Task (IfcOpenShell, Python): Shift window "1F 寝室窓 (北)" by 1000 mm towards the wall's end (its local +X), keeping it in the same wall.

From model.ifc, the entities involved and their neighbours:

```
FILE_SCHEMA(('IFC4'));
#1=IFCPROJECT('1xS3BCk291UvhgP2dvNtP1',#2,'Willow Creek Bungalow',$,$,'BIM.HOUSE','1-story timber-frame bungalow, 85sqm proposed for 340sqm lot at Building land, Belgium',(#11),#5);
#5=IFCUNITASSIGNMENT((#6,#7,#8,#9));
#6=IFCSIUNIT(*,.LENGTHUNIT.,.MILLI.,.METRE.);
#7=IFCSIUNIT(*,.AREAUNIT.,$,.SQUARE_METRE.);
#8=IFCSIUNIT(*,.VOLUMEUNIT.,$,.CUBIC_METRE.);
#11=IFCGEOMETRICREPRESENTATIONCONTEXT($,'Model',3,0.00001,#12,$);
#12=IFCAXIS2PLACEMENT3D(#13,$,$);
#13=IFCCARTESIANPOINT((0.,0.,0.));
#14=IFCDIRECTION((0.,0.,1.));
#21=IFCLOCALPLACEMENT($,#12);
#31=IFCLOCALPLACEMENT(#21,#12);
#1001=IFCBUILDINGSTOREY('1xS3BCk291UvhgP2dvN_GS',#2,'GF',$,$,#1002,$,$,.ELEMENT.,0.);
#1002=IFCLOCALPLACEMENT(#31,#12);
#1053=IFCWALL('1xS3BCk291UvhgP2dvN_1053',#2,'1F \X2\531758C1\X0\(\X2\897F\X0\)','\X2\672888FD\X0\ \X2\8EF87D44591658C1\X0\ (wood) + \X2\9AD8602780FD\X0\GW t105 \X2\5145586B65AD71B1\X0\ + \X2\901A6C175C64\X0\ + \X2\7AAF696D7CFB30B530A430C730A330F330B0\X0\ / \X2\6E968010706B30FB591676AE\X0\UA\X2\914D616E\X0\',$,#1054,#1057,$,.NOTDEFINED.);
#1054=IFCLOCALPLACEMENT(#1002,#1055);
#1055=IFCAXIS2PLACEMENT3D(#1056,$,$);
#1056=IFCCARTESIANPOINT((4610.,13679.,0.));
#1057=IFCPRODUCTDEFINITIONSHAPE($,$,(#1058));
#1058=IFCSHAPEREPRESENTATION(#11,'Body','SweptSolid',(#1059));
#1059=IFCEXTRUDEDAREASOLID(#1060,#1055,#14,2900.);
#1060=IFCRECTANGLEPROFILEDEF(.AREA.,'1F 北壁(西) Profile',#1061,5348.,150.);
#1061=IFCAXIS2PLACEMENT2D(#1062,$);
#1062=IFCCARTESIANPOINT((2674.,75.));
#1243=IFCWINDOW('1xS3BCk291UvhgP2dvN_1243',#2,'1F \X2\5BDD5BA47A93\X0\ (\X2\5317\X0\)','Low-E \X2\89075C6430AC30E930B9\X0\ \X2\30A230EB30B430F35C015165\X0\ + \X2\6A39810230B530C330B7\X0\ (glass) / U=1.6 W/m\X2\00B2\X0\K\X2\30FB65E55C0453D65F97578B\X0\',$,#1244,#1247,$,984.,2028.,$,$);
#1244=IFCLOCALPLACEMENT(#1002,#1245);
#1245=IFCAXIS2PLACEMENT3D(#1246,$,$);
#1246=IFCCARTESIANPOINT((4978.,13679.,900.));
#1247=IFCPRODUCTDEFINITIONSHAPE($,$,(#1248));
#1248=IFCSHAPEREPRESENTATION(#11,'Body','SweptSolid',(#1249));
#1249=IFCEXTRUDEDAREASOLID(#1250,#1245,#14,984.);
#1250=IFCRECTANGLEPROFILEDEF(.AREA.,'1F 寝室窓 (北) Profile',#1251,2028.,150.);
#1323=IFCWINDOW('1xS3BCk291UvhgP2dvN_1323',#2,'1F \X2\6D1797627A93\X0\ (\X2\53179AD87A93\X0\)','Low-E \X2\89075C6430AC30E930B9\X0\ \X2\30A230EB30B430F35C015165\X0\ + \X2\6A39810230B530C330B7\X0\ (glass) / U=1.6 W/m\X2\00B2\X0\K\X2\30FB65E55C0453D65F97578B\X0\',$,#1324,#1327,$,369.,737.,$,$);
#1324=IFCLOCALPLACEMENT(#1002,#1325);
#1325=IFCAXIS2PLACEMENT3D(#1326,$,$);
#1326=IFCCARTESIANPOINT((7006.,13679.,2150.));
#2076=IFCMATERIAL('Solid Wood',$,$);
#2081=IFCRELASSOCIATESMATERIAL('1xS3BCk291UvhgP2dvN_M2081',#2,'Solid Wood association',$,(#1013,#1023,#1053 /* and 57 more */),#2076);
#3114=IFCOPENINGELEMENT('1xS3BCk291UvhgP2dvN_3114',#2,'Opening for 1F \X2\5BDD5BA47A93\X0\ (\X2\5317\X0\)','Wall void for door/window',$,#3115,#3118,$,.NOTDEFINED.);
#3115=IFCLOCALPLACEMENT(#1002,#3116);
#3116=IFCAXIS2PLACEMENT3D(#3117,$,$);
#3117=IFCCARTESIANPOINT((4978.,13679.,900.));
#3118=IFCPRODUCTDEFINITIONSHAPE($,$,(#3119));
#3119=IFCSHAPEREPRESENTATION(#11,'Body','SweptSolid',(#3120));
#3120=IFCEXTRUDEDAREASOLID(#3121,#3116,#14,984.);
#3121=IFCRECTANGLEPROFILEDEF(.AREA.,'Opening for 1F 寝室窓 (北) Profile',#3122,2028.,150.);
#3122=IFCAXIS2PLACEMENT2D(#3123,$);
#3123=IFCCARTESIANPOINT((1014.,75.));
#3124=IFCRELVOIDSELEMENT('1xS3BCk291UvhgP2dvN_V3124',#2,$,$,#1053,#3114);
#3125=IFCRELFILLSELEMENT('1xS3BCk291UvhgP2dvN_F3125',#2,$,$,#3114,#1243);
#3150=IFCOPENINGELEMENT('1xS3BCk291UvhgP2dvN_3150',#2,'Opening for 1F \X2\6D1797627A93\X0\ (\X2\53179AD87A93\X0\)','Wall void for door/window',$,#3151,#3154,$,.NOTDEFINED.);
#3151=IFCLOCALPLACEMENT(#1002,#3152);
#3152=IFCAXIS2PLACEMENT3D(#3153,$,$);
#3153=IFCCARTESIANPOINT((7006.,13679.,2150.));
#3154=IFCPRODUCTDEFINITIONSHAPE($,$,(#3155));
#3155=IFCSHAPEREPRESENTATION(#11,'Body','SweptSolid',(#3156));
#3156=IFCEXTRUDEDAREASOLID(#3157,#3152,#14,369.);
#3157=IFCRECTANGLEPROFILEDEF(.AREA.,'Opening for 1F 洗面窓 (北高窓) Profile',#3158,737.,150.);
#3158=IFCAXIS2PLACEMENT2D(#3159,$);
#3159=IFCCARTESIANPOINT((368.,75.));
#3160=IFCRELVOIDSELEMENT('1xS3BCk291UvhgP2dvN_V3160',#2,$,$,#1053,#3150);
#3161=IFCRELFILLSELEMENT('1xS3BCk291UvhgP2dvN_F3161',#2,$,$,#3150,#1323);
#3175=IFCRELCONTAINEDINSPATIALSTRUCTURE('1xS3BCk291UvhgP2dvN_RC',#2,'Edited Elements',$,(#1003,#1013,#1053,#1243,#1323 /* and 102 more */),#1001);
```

```python
import ifcopenshell
import ifcopenshell.api.geometry
import ifcopenshell.util.placement

model = ifcopenshell.open("model.ifc")

window = model.by_guid("1xS3BCk291UvhgP2dvN_1243")
opening = window.FillsVoids[0].RelatingOpeningElement
wall = opening.VoidsElements[0].RelatingBuildingElement

wall_matrix = ifcopenshell.util.placement.get_local_placement(wall.ObjectPlacement)
shift = wall_matrix[:3, 0] * 1000.0
before = ifcopenshell.util.placement.get_local_placement(window.ObjectPlacement)[:3, 3].copy()

# The window is not placed relative to its opening, so move both.
for product in (opening, window):
    matrix = ifcopenshell.util.placement.get_local_placement(product.ObjectPlacement)
    matrix[:3, 3] += shift
    ifcopenshell.api.geometry.edit_object_placement(model, product=product, matrix=matrix, is_si=False)

after = ifcopenshell.util.placement.get_local_placement(window.ObjectPlacement)[:3, 3]
print("window moved by", (after - before).round(3) + 0.0)

model.write("model_edited.ifc")
```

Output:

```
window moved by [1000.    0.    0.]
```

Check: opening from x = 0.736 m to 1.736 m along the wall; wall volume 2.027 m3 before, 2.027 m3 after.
